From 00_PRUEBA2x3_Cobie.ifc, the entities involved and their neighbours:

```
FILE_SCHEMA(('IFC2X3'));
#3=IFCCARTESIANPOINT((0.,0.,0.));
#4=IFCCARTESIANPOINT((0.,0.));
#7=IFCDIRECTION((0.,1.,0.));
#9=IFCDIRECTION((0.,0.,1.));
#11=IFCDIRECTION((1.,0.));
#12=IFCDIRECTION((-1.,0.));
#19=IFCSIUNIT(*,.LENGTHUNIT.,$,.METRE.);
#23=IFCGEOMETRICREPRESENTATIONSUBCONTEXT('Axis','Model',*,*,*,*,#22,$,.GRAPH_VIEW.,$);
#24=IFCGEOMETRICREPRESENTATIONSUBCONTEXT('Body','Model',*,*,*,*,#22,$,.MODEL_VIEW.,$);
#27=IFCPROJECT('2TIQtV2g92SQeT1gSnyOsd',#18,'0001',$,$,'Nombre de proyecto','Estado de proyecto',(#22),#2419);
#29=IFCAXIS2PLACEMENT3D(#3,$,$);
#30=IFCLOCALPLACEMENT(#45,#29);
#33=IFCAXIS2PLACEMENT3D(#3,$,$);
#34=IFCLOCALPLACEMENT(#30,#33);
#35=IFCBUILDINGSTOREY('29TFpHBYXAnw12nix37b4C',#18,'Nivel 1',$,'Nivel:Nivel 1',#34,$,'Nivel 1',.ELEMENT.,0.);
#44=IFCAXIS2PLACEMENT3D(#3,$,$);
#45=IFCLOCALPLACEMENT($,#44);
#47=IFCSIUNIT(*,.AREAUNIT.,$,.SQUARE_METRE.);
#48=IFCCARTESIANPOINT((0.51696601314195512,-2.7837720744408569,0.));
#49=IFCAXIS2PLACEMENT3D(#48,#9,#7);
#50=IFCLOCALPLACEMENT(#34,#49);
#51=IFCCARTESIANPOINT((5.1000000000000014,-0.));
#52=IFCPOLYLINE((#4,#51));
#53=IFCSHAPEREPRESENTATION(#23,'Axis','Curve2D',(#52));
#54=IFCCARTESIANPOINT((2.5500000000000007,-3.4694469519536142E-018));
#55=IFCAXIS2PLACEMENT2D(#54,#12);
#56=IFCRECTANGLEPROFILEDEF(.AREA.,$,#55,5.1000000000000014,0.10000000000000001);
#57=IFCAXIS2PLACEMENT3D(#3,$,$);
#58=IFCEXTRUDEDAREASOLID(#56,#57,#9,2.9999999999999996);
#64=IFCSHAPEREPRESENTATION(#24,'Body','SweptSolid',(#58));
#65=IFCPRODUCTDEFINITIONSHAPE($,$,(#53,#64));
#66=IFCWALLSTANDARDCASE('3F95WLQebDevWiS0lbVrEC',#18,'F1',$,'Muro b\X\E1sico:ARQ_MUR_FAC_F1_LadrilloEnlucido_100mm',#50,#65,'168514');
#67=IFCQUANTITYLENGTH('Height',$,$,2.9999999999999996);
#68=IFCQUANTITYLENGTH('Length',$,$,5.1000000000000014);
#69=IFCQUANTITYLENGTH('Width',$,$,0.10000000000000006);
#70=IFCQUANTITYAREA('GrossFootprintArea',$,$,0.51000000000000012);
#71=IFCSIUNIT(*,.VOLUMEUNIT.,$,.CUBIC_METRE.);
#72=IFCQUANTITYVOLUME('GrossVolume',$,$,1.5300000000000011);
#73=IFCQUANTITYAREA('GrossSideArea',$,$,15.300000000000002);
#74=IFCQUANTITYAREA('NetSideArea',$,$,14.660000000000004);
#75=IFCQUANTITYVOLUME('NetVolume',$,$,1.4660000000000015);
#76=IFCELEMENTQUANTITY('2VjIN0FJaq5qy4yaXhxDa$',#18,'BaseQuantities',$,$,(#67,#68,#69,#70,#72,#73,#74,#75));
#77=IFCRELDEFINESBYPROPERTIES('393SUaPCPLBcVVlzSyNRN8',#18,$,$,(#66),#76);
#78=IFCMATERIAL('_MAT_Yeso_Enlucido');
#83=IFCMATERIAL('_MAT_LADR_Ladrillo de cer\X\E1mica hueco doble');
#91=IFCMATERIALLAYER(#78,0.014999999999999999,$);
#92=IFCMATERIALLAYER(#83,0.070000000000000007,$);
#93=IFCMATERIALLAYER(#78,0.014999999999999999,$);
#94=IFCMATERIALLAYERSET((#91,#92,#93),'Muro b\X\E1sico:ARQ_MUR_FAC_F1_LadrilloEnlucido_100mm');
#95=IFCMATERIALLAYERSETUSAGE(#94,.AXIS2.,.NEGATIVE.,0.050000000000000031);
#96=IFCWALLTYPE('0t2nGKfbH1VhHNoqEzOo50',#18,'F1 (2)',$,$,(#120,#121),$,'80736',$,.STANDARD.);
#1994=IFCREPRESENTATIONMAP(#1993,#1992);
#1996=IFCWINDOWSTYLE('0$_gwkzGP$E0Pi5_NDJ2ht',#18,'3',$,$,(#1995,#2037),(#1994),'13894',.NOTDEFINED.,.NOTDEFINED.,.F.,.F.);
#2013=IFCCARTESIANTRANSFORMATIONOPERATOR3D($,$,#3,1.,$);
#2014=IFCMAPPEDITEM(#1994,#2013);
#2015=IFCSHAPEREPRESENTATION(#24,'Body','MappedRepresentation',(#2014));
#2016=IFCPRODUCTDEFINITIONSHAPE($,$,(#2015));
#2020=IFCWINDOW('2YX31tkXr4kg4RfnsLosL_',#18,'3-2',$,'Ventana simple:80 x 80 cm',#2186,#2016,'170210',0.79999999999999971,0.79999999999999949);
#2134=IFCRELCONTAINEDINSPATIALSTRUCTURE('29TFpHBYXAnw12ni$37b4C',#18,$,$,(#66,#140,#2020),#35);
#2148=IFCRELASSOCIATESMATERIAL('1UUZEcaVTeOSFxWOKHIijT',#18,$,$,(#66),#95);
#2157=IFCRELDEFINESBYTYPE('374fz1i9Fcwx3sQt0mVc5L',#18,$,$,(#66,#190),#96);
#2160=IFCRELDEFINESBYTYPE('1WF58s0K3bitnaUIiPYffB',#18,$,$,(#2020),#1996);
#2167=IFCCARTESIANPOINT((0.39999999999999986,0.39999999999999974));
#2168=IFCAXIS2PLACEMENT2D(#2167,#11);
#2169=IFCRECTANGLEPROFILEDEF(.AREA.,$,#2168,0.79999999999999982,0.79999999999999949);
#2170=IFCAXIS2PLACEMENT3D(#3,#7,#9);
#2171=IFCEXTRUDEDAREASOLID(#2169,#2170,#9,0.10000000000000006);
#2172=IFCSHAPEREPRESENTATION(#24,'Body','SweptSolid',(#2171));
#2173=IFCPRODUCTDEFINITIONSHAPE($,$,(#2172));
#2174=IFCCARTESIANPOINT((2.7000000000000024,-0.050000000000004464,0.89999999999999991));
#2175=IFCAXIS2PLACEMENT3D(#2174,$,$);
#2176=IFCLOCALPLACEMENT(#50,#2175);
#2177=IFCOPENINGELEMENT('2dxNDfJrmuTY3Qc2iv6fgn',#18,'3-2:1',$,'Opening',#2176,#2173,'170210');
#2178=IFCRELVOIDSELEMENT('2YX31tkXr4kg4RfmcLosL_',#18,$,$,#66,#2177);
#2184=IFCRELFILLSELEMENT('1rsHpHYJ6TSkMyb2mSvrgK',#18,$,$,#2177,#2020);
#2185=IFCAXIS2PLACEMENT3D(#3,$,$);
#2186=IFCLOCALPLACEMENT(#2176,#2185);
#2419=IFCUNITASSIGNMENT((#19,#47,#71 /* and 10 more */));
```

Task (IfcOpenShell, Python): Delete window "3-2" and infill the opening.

```python
import ifcopenshell
import ifcopenshell.api.feature
import ifcopenshell.api.pset
import ifcopenshell.api.root
import ifcopenshell.geom
import ifcopenshell.util.element
import ifcopenshell.util.shape
import ifcopenshell.util.unit

model = ifcopenshell.open("00_PRUEBA2x3_Cobie.ifc")
area_scale = ifcopenshell.util.unit.calculate_unit_scale(model, "AREAUNIT")
volume_scale = ifcopenshell.util.unit.calculate_unit_scale(model, "VOLUMEUNIT")
settings = ifcopenshell.geom.settings()


def volume(element):
    """Net volume in cubic metres, openings subtracted."""
    shape = ifcopenshell.geom.create_shape(settings, element)
    return ifcopenshell.util.shape.get_volume(shape.geometry)


window = model.by_id(2020)
opening = window.FillsVoids[0].RelatingOpeningElement
wall = opening.VoidsElements[0].RelatingBuildingElement
before = volume(wall)

ifcopenshell.api.root.remove_product(model, product=window)
ifcopenshell.api.feature.remove_feature(model, feature=opening)

after = volume(wall)
thickness = 0.1  # wall thickness in metres

# Update the wall's stored quantities.
qto = model.by_id(ifcopenshell.util.element.get_pset(wall, "BaseQuantities", should_inherit=False)["id"])
ifcopenshell.api.pset.edit_qto(model, qto=qto, properties={
    "NetSideArea": after / thickness / area_scale,
    "NetVolume": after / volume_scale,
})

print(f"wall volume {before:.3f} -> {after:.3f} m3")

model.write("00_PRUEBA2x3_Cobie_v2.ifc")
```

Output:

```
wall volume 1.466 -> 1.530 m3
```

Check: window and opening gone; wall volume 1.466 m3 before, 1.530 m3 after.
